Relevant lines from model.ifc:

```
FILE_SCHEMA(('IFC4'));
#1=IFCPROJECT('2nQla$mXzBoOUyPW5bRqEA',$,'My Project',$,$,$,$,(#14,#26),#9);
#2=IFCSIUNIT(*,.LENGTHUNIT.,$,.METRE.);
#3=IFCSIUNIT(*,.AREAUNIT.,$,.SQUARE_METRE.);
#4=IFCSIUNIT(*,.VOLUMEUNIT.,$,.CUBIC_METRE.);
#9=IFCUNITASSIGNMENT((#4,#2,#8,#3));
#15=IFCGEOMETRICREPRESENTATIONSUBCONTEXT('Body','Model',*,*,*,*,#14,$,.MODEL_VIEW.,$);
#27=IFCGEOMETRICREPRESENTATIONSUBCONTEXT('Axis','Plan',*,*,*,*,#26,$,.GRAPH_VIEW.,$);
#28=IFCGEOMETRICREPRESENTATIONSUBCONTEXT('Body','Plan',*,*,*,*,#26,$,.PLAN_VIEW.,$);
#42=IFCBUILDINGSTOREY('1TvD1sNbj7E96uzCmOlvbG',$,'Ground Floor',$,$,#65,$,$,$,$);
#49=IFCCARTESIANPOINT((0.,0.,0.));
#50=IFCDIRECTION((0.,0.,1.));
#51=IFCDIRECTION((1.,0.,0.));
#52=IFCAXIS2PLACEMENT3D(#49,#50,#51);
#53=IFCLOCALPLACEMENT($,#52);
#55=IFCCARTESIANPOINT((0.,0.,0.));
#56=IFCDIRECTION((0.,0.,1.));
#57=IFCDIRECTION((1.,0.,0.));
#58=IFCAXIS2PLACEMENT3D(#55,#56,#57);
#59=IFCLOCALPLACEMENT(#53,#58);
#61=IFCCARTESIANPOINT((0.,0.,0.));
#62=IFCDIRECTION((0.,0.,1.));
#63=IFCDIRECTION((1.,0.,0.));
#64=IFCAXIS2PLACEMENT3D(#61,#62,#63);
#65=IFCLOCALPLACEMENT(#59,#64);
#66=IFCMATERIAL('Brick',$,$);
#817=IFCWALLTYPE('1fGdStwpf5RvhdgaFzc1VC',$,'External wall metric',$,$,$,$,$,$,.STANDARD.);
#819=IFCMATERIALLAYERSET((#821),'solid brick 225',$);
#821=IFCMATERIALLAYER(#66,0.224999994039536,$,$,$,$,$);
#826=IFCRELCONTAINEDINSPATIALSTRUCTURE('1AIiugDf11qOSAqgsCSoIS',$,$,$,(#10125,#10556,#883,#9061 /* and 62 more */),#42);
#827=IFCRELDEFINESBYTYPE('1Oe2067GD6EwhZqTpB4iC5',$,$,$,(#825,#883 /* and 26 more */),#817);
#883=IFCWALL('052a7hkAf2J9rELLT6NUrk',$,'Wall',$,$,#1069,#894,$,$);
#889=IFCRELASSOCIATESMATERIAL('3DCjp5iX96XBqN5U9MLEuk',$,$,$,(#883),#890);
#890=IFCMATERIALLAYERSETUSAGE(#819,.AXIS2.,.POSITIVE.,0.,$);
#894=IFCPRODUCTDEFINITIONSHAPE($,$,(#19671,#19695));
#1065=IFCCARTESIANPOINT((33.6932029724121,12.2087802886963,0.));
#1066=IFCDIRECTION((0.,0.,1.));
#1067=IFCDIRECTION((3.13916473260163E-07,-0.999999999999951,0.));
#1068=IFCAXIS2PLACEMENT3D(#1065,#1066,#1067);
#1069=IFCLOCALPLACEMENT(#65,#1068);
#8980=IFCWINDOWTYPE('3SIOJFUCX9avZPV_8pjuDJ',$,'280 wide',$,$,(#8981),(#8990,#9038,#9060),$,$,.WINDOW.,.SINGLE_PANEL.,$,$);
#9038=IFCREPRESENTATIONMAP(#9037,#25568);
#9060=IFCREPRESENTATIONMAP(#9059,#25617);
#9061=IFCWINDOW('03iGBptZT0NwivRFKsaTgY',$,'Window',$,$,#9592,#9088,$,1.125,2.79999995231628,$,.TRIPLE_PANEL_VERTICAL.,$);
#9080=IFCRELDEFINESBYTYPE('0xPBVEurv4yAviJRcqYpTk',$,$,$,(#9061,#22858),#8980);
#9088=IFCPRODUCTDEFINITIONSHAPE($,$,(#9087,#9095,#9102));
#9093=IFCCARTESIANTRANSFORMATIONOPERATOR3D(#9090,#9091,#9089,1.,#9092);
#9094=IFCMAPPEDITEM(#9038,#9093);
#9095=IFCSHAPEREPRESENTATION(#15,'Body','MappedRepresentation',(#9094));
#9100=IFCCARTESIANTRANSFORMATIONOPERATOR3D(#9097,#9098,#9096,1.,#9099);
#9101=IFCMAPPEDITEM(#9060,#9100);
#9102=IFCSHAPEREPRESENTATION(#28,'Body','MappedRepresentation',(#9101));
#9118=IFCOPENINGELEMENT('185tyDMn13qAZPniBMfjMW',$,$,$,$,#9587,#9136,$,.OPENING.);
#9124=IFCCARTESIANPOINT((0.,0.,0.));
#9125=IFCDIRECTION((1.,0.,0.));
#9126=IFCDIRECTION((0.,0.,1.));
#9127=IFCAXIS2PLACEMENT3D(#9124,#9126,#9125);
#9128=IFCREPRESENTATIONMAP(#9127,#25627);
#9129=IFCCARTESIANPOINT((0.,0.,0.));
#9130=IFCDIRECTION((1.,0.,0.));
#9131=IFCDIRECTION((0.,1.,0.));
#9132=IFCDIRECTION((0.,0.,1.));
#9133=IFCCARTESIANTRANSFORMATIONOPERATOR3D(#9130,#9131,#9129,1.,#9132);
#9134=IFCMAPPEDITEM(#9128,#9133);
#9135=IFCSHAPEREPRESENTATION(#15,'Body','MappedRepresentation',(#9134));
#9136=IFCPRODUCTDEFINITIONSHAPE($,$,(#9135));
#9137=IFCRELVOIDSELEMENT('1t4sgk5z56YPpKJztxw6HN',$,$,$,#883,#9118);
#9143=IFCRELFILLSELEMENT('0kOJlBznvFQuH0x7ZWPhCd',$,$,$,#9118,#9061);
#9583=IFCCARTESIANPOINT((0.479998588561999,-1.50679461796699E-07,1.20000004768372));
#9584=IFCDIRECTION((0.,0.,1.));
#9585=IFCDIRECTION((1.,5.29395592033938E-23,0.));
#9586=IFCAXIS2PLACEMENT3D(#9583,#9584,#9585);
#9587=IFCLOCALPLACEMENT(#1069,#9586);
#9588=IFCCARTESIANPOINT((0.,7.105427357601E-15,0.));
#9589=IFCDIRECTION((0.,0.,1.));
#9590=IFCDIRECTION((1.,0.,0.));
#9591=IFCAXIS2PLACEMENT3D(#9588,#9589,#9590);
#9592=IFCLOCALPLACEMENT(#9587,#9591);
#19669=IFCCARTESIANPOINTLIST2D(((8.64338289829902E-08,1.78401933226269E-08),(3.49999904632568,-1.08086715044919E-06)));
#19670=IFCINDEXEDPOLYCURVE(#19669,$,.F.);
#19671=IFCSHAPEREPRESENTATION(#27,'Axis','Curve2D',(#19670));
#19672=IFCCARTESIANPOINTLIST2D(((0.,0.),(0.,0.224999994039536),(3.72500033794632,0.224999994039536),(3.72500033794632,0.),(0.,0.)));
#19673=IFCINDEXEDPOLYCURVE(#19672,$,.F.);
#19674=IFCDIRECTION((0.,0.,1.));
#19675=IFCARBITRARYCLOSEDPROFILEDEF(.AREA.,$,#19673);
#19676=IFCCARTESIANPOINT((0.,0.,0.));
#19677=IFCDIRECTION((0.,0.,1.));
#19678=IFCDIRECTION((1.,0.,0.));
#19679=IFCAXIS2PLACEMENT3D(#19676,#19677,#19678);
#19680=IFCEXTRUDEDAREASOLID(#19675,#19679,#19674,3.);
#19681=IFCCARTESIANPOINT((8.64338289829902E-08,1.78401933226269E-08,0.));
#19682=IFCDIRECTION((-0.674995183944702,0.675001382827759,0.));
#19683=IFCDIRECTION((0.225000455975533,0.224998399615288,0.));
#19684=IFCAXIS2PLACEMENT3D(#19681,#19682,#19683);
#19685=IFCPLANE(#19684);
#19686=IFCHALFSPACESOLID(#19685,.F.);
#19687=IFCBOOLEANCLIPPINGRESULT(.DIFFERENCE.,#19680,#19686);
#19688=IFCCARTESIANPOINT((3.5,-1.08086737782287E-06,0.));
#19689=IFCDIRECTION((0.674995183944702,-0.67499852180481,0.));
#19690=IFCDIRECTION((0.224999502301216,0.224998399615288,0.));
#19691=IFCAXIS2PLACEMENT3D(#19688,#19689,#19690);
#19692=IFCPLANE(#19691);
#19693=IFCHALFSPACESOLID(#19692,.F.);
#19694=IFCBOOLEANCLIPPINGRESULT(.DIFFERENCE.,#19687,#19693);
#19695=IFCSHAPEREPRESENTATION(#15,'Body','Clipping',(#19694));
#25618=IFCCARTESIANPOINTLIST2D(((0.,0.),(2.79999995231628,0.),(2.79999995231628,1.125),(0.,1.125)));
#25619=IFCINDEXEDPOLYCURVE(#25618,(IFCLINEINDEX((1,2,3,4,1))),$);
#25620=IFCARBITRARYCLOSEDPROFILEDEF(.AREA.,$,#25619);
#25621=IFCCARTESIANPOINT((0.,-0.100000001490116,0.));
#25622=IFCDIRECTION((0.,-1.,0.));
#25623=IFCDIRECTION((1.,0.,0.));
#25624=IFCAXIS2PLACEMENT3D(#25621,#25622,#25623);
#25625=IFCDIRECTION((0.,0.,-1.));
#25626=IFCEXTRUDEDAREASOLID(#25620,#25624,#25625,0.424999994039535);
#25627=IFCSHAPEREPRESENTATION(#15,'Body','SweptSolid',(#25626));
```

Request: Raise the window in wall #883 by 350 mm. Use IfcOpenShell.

```python
import numpy as np
import ifcopenshell
import ifcopenshell.api.geometry
import ifcopenshell.util.placement
import ifcopenshell.util.unit

model = ifcopenshell.open("model.ifc")
unit_scale = ifcopenshell.util.unit.calculate_unit_scale(model)

window = model.by_guid("03iGBptZT0NwivRFKsaTgY")
opening = window.FillsVoids[0].RelatingOpeningElement
dz = 0.35 / unit_scale

shift = np.array([0.0, 0.0, dz])
# The window is placed relative to its opening, so it follows when the opening moves.
matrix = ifcopenshell.util.placement.get_local_placement(opening.ObjectPlacement)
matrix[:3, 3] += shift
ifcopenshell.api.geometry.edit_object_placement(
    model, product=opening, matrix=matrix, is_si=False, should_transform_children=True
)

print(f"moved by {dz * unit_scale:+.3f} m")

model.write("model_edited.ifc")
```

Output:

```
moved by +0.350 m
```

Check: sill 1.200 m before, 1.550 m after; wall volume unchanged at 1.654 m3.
